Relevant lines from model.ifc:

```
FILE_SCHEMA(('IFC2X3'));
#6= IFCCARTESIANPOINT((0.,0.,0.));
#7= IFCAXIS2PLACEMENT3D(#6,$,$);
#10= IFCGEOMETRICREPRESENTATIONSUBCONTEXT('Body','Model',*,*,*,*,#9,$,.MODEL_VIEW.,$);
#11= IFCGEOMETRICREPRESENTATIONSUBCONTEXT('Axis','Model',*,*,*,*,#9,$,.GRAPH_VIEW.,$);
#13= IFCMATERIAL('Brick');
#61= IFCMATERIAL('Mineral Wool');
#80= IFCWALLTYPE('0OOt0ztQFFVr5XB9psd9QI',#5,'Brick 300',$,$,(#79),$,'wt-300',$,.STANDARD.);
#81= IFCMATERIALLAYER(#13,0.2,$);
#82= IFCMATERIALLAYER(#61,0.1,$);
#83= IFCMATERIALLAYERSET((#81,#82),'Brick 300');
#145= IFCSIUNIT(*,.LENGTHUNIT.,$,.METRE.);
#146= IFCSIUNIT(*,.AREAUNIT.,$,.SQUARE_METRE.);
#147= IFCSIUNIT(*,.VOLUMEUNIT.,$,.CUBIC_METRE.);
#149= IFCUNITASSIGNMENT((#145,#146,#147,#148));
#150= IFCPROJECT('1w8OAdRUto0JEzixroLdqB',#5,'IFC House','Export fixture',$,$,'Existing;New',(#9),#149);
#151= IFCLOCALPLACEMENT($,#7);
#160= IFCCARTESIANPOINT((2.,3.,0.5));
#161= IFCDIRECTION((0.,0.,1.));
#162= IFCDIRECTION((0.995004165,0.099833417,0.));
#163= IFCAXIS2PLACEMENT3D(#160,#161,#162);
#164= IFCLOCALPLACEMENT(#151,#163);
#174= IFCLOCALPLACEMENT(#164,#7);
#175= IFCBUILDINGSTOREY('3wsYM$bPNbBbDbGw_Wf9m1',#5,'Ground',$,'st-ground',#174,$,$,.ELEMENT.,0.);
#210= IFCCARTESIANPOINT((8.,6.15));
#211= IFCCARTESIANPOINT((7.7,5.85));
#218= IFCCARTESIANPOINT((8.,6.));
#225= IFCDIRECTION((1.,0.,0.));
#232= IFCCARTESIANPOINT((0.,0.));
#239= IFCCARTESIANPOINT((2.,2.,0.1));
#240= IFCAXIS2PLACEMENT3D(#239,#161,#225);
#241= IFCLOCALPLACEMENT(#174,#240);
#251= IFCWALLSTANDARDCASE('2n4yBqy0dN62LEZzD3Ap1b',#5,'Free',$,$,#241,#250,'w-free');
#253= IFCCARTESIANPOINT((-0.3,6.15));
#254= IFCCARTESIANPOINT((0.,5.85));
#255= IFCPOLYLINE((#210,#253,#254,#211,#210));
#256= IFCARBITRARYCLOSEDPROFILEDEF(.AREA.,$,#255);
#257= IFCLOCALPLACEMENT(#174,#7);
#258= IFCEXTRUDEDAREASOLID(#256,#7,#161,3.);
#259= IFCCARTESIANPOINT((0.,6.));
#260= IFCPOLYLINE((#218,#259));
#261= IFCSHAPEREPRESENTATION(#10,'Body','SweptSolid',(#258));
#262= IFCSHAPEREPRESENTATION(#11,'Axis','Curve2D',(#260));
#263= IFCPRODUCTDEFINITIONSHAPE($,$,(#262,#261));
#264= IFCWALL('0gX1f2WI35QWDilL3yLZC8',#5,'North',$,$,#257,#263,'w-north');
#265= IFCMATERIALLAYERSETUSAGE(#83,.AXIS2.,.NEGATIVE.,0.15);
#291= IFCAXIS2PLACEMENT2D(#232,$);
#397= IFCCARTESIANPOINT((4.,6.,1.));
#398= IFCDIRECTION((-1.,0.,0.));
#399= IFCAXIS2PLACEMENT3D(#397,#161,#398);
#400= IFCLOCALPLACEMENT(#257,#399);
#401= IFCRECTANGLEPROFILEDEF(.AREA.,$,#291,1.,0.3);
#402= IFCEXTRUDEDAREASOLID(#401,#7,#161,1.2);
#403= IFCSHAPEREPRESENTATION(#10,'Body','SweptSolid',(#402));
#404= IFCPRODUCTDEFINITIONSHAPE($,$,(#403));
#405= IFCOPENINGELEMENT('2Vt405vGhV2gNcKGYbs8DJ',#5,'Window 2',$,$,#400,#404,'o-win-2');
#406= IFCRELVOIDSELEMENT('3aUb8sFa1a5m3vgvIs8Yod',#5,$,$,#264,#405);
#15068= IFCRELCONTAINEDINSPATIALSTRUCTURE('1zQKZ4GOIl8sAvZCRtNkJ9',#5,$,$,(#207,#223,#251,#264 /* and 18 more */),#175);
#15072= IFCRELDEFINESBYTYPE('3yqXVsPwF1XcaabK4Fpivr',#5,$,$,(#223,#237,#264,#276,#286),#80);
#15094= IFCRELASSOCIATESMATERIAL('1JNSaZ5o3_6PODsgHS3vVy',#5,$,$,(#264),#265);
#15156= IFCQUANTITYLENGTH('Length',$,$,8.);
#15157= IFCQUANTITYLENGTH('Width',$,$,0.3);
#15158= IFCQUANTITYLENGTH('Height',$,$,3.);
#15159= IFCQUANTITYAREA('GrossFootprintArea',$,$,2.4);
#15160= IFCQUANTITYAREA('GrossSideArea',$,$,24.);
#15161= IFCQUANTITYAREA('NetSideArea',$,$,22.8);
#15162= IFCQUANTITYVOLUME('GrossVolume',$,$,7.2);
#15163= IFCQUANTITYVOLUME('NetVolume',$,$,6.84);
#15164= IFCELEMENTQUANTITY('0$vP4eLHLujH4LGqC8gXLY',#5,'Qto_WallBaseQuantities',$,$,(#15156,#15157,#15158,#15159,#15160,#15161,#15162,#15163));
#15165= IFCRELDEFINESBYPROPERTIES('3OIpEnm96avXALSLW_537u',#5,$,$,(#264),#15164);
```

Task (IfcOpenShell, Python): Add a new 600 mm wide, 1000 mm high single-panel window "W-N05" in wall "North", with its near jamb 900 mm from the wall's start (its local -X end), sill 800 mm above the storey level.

```python
import numpy as np
import ifcopenshell
import ifcopenshell.api.feature
import ifcopenshell.api.geometry
import ifcopenshell.api.pset
import ifcopenshell.api.root
import ifcopenshell.api.spatial
import ifcopenshell.api.type
import ifcopenshell.geom
import ifcopenshell.util.element
import ifcopenshell.util.placement
import ifcopenshell.util.representation
import ifcopenshell.util.shape
import ifcopenshell.util.unit

model = ifcopenshell.open("model.ifc")
unit_scale = ifcopenshell.util.unit.calculate_unit_scale(model)
area_scale = ifcopenshell.util.unit.calculate_unit_scale(model, "AREAUNIT")
volume_scale = ifcopenshell.util.unit.calculate_unit_scale(model, "VOLUMEUNIT")
settings = ifcopenshell.geom.settings()


def volume(element):
    """Net volume in cubic metres, openings subtracted."""
    shape = ifcopenshell.geom.create_shape(settings, element)
    return ifcopenshell.util.shape.get_volume(shape.geometry)


wall = model.by_guid("0gX1f2WI35QWDilL3yLZC8")
storey = ifcopenshell.util.element.get_container(wall, ifc_class="IfcBuildingStorey")
context = ifcopenshell.util.representation.get_context(model, "Model", "Body", "MODEL_VIEW")
before = volume(wall)

width, height, from_end, sill = 0.6, 1, 0.9, 0.8  # metres

# The wall runs along its own X axis, and the end named is its -X end.
wall_shape = ifcopenshell.geom.create_shape(settings, wall)
x, y, z = ifcopenshell.util.shape.get_vertices(wall_shape.geometry).T
start = x.min() + from_end
face, thickness = float(y.min()), float(y.max() - y.min())
wall_matrix = ifcopenshell.util.placement.get_local_placement(wall.ObjectPlacement)
level = ifcopenshell.util.placement.get_local_placement(storey.ObjectPlacement)[2, 3]


def in_wall(x, y):
    """Placement at x, y metres in the wall's axes, at sill height."""
    matrix = wall_matrix.copy()
    matrix[:, 3] = wall_matrix @ np.array([x / unit_scale, y / unit_scale, 0.0, 1.0])
    matrix[2, 3] = level + sill / unit_scale
    return matrix


# Opening: a box that overshoots both wall faces by 50 mm.
opening = ifcopenshell.api.root.create_entity(model, ifc_class="IfcOpeningElement")
box = ifcopenshell.api.geometry.add_wall_representation(
    model, context=context, length=width, height=height, thickness=thickness + 0.1
)
ifcopenshell.api.geometry.assign_representation(model, product=opening, representation=box)
ifcopenshell.api.geometry.edit_object_placement(model, product=opening, matrix=in_wall(start, face - 0.05), is_si=False)
ifcopenshell.api.feature.add_feature(model, feature=opening, element=wall)

window = ifcopenshell.api.root.create_entity(model, ifc_class="IfcWindow", name="W-N05")
window.OverallWidth, window.OverallHeight = width / unit_scale, height / unit_scale
body = ifcopenshell.api.geometry.add_window_representation(
    model,
    context=context,
    overall_width=window.OverallWidth,
    overall_height=window.OverallHeight,
    partition_type="SINGLE_PANEL",
)
ifcopenshell.api.geometry.assign_representation(model, product=window, representation=body)
ifcopenshell.api.spatial.assign_container(model, products=[window], relating_structure=storey)
fills = ifcopenshell.api.feature.add_filling(model, opening=opening, element=window)
fills.OwnerHistory = window.OwnerHistory  # required in IFC2X3

# IFC2X3 keeps the operation on the window style.
style = ifcopenshell.api.root.create_entity(model, ifc_class="IfcWindowStyle", name="W-N05")
style.OperationType, style.ConstructionType = "SINGLE_PANEL", "NOTDEFINED"
style.ParameterTakesPrecedence = style.Sizeable = False
ifcopenshell.api.type.assign_type(model, related_objects=[window], relating_type=style)

# Centre the window in the wall's thickness.
ifcopenshell.api.geometry.edit_object_placement(model, product=window, matrix=in_wall(start, face), is_si=False)
window_shape = ifcopenshell.geom.create_shape(settings, window)
depth = ifcopenshell.util.shape.get_vertices(window_shape.geometry)[:, 1]
offset = face + thickness / 2 - (depth.min() + depth.max()) / 2
ifcopenshell.api.geometry.edit_object_placement(model, product=window, matrix=in_wall(start, offset), is_si=False)

after = volume(wall)

# Update the wall's stored quantities.
qto = model.by_id(ifcopenshell.util.element.get_pset(wall, "Qto_WallBaseQuantities", should_inherit=False)["id"])
ifcopenshell.api.pset.edit_qto(model, qto=qto, properties={
    "NetSideArea": after / thickness / area_scale,
    "NetVolume": after / volume_scale,
})

print(f"wall volume {before:.3f} -> {after:.3f} m3")

model.write("model_v2.ifc")
```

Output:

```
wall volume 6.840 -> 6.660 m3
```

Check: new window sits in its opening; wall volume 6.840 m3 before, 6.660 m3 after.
